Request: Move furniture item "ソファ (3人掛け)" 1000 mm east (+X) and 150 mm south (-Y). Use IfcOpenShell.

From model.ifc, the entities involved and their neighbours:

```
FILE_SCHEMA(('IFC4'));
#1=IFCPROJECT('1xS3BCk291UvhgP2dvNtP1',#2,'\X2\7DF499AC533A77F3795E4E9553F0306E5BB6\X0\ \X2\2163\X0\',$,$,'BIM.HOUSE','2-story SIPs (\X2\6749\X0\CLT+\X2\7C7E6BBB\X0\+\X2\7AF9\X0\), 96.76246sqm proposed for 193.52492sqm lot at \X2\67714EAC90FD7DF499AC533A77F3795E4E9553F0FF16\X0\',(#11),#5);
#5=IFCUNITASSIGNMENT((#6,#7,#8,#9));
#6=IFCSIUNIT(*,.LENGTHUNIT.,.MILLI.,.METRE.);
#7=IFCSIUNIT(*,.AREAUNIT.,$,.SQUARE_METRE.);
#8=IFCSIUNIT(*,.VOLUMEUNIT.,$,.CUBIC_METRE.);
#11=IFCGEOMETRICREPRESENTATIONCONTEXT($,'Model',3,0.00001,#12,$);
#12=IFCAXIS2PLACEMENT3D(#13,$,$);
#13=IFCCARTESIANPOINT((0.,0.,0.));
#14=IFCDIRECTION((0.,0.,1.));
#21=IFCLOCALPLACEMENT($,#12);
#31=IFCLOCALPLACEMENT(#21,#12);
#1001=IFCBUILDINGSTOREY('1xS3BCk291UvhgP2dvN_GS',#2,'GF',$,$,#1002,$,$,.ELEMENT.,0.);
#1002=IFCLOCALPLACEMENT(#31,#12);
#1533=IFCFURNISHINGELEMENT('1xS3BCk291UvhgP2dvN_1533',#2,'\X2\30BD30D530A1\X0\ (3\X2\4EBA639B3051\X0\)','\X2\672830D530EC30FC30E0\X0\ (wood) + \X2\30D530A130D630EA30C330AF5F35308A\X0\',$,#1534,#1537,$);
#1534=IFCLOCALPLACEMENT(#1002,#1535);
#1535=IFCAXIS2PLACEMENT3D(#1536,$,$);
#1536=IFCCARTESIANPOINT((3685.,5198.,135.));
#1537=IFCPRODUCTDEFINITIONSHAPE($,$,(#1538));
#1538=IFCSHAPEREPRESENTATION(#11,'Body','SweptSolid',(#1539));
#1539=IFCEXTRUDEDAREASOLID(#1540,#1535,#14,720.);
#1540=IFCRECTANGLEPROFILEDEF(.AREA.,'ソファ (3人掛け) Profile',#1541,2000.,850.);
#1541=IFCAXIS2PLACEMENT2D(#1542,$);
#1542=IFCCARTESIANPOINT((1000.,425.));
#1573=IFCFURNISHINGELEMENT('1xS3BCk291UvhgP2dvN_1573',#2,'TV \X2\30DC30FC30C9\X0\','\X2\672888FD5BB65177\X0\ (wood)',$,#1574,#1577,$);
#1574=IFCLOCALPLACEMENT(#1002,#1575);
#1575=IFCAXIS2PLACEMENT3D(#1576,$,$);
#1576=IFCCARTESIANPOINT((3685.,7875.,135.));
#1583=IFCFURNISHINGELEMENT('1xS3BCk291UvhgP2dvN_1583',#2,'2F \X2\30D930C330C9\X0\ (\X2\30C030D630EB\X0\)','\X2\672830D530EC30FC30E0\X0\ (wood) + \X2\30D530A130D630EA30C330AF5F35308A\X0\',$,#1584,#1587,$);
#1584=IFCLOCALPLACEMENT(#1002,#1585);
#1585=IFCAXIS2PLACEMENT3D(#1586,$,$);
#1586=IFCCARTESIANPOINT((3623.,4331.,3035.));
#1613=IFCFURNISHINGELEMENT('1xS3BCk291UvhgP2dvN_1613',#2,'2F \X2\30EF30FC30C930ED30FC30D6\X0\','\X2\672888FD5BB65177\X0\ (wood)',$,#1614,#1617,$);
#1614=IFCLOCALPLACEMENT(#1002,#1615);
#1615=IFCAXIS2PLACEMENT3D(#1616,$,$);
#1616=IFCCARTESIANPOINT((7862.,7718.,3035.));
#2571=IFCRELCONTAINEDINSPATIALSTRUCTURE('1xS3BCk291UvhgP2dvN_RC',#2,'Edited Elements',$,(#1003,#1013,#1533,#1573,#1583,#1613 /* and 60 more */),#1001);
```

```python
import ifcopenshell
import ifcopenshell.api.geometry
import ifcopenshell.util.placement

model = ifcopenshell.open("model.ifc")

item = model.by_id(1533)
matrix = ifcopenshell.util.placement.get_local_placement(item.ObjectPlacement)
matrix[0, 3] += 1000.0
matrix[1, 3] -= 150.0
ifcopenshell.api.geometry.edit_object_placement(model, product=item, matrix=matrix, is_si=False)

print(ifcopenshell.util.placement.get_local_placement(item.ObjectPlacement).round(3) + 0.0)

model.write("model_v2.ifc")
```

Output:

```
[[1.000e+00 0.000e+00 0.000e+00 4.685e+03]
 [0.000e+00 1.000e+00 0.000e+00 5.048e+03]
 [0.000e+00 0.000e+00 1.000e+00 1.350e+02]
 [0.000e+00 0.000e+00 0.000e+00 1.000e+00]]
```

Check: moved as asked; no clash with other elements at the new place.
